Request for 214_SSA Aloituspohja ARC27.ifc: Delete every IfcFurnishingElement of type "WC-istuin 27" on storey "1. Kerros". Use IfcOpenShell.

First a look at what the model holds.

```python
import ifcopenshell
import ifcopenshell.util.element

model = ifcopenshell.open("214_SSA Aloituspohja ARC27.ifc")
print(model.schema)
storey = next(s for s in model.by_type("IfcBuildingStorey") if s.Name == "1. Kerros")
furniture = [e for e in ifcopenshell.util.element.get_decomposition(storey) if e.is_a("IfcFurnishingElement")]
seen = {}
for e in furniture:
    element_type = ifcopenshell.util.element.get_type(e)
    name = element_type.Name if element_type not in (None, e) else None
    seen[name] = seen.get(name, 0) + 1
for name, count in sorted(seen.items(), key=str):
    print(count, "x", name)
```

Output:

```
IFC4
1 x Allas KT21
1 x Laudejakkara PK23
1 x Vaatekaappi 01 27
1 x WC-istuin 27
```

```python
import ifcopenshell
import ifcopenshell.api.root
import ifcopenshell.util.element

model = ifcopenshell.open("214_SSA Aloituspohja ARC27.ifc")

storey = next(s for s in model.by_type("IfcBuildingStorey") if s.Name == "1. Kerros")
furniture = [e for e in ifcopenshell.util.element.get_decomposition(storey) if e.is_a("IfcFurnishingElement")]
targets = [e for e in furniture if (t := ifcopenshell.util.element.get_type(e)) not in (None, e) and t.Name == "WC-istuin 27"]

for e in targets:
    ifcopenshell.api.root.remove_product(model, product=e)
print(len(targets), "removed")

model.write("214_SSA Aloituspohja ARC27_v2.ifc")
```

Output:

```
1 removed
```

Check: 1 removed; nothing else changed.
